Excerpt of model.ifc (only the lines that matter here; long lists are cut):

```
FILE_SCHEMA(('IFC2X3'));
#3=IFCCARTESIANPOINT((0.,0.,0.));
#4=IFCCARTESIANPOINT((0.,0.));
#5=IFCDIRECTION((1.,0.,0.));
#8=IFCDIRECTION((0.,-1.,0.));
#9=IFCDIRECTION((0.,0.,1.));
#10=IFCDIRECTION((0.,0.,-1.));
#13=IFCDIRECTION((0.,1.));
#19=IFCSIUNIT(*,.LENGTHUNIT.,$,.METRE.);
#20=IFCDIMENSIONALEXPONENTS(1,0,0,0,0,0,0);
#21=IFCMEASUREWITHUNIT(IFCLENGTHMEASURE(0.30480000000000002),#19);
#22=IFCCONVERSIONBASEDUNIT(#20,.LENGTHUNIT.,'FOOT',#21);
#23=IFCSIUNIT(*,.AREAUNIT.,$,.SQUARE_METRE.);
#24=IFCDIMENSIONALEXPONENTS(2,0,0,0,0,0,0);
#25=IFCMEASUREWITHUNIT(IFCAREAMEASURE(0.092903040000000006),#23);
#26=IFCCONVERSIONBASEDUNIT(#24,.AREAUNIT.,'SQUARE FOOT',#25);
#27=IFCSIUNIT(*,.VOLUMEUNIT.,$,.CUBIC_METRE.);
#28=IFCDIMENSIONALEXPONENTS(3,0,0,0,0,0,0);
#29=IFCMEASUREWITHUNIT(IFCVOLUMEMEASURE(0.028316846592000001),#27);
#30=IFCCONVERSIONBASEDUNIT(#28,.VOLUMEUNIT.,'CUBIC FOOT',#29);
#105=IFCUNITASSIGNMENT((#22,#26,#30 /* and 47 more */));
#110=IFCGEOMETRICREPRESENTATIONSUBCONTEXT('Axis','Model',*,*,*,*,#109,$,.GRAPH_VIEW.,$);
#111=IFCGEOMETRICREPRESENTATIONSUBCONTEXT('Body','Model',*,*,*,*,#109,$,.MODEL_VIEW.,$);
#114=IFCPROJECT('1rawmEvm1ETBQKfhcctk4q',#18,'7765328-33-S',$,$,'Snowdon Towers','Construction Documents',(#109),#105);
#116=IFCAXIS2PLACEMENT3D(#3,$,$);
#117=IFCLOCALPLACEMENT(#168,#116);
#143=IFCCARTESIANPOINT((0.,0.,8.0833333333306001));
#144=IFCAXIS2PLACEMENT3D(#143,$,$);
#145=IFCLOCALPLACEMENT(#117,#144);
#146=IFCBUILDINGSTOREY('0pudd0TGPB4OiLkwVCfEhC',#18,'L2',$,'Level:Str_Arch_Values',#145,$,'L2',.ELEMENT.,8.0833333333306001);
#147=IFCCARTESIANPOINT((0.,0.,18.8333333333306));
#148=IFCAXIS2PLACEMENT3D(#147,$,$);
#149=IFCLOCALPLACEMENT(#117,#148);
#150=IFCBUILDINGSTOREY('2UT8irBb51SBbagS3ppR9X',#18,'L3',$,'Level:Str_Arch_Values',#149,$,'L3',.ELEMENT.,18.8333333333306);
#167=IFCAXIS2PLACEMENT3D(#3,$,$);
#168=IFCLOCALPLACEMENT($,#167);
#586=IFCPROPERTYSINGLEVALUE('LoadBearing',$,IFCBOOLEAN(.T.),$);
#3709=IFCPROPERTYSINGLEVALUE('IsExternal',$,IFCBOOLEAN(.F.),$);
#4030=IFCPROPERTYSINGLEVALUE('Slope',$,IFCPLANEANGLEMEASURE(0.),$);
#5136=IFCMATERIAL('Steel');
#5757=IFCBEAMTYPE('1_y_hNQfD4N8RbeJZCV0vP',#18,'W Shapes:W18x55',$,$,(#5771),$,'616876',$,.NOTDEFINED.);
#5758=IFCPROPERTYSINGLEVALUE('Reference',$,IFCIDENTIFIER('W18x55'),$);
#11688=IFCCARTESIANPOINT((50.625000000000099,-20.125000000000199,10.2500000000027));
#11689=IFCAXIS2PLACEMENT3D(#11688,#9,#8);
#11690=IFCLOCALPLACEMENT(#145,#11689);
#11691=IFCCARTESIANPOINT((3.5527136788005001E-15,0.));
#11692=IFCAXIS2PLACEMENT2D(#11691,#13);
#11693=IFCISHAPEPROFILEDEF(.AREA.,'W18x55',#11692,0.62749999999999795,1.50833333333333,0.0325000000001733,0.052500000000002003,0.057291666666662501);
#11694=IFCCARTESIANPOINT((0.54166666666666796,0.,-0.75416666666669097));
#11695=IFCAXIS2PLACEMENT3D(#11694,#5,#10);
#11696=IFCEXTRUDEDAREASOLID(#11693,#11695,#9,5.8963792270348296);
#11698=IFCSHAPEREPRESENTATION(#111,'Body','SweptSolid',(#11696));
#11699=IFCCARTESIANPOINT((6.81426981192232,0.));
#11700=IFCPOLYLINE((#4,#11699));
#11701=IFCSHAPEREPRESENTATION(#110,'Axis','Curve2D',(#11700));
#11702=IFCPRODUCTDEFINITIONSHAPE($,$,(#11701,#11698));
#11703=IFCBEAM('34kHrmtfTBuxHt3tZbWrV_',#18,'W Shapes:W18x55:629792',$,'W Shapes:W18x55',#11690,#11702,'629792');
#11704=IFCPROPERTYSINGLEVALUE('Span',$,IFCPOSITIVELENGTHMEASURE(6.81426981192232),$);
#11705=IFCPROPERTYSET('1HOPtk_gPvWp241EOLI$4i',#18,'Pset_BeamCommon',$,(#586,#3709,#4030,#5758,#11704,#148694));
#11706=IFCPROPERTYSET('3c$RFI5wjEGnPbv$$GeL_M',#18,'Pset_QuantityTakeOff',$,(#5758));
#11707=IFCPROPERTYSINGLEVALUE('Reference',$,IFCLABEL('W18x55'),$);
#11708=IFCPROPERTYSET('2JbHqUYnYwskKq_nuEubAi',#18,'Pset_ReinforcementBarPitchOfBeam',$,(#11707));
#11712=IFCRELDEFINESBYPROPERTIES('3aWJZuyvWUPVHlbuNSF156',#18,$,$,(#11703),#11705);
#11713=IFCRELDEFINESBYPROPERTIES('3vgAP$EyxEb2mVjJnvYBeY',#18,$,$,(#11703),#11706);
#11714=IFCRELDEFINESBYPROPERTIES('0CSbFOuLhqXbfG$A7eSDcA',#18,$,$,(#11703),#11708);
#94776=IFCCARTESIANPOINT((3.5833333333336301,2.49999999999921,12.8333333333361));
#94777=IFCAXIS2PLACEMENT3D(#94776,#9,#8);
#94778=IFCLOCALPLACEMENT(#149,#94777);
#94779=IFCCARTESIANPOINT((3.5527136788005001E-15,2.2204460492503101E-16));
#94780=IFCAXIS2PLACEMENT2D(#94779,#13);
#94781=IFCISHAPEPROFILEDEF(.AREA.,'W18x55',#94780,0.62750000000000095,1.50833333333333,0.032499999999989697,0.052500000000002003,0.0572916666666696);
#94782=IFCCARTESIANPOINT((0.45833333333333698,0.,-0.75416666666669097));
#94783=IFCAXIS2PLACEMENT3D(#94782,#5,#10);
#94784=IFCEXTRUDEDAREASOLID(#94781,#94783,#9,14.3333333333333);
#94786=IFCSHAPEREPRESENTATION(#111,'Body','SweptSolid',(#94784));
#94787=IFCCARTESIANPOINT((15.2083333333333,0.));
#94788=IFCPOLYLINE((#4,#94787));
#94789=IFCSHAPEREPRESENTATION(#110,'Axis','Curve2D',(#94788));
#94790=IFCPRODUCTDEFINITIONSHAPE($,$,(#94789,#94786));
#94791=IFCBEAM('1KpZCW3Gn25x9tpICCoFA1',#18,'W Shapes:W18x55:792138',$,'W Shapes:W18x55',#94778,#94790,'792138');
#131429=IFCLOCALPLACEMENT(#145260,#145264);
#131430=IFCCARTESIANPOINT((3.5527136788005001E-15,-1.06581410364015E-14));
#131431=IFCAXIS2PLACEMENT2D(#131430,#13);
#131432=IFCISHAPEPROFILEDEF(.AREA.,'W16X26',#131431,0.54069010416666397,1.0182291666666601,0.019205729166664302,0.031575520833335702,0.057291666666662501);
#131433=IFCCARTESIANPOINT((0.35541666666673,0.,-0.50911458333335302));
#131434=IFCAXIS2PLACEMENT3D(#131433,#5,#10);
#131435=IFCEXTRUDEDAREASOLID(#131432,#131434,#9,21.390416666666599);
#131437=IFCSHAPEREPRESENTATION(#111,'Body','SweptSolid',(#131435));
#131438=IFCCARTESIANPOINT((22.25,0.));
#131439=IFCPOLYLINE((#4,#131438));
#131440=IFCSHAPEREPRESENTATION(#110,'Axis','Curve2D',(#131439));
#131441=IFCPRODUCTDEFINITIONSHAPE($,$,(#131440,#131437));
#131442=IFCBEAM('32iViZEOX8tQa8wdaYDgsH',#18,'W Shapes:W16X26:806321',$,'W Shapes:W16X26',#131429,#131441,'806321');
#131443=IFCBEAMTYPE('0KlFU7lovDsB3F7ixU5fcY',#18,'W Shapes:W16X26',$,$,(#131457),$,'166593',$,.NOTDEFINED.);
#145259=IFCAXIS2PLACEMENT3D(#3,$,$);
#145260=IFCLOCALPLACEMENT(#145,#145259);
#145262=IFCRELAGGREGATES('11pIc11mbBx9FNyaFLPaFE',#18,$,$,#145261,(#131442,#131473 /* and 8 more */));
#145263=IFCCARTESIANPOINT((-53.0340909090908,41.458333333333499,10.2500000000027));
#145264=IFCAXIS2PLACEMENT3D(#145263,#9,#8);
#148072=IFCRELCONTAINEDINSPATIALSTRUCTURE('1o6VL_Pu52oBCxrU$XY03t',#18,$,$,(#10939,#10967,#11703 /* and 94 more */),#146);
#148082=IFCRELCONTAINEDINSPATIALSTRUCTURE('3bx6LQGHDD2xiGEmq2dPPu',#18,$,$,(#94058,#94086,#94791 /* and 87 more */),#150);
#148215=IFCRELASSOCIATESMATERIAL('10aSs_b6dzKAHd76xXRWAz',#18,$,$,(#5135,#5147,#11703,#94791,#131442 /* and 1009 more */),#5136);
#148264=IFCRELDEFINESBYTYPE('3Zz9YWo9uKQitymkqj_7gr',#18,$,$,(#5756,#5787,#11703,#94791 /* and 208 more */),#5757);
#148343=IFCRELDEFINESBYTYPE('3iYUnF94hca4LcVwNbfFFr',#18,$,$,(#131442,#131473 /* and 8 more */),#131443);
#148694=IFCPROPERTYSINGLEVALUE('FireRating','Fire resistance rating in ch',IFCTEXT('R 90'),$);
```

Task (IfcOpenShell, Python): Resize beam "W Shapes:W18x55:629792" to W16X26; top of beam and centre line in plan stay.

```python
import ifcopenshell
import ifcopenshell.api.pset
import ifcopenshell.api.type
import ifcopenshell.util.element
import ifcopenshell.util.representation

model = ifcopenshell.open("model.ifc")

member = model.by_guid("34kHrmtfTBuxHt3tZbWrV_")
source = next(p for p in model.by_type("IfcIShapeProfileDef") if p.ProfileName == "W16X26")

body = ifcopenshell.util.representation.get_representation(member, "Model", "Body")
solid = body.Items[0]
old_profile = solid.SweptArea

# Copy the section's sizes but keep this member's own profile position.
profile = ifcopenshell.util.element.copy(model, source)
# Profiles are centred, so shift by half the change in depth to hold the top.
shift = (old_profile.OverallDepth - profile.OverallDepth) / 2
x, y = old_profile.Position.Location.Coordinates
up = (-1.0, 0.0)  # upwards, in the solid's own plane
location = model.createIfcCartesianPoint((x + up[0] * shift, y + up[1] * shift))
profile.Position = model.createIfcAxis2Placement2D(location, old_profile.Position.RefDirection)
solid.SweptArea = profile
if not model.get_total_inverses(old_profile):
    ifcopenshell.util.element.remove_deep2(model, old_profile)

new_type = model.by_guid("0KlFU7lovDsB3F7ixU5fcY")
ifcopenshell.api.type.assign_type(
    model, related_objects=[member], relating_type=new_type, should_map_representations=False
)
member.Name = member.Name.replace("W18x55", "W16X26")
member.ObjectType = "W Shapes:W16X26"
pset = model.by_id(ifcopenshell.util.element.get_pset(member, "Pset_BeamCommon", should_inherit=False)["id"])
ifcopenshell.api.pset.edit_pset(model, pset=pset, properties={"Reference": "W16X26"})
pset = model.by_id(ifcopenshell.util.element.get_pset(member, "Pset_QuantityTakeOff", should_inherit=False)["id"])
ifcopenshell.api.pset.edit_pset(model, pset=pset, properties={"Reference": "W16X26"})
pset = model.by_id(ifcopenshell.util.element.get_pset(member, "Pset_ReinforcementBarPitchOfBeam", should_inherit=False)["id"])
ifcopenshell.api.pset.edit_pset(model, pset=pset, properties={"Reference": "W16X26"})

print(solid.SweptArea)

model.write("model_rev.ifc")
```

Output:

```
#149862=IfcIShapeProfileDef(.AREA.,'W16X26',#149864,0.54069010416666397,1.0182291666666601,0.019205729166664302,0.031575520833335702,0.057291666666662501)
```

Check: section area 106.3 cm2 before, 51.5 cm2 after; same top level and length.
